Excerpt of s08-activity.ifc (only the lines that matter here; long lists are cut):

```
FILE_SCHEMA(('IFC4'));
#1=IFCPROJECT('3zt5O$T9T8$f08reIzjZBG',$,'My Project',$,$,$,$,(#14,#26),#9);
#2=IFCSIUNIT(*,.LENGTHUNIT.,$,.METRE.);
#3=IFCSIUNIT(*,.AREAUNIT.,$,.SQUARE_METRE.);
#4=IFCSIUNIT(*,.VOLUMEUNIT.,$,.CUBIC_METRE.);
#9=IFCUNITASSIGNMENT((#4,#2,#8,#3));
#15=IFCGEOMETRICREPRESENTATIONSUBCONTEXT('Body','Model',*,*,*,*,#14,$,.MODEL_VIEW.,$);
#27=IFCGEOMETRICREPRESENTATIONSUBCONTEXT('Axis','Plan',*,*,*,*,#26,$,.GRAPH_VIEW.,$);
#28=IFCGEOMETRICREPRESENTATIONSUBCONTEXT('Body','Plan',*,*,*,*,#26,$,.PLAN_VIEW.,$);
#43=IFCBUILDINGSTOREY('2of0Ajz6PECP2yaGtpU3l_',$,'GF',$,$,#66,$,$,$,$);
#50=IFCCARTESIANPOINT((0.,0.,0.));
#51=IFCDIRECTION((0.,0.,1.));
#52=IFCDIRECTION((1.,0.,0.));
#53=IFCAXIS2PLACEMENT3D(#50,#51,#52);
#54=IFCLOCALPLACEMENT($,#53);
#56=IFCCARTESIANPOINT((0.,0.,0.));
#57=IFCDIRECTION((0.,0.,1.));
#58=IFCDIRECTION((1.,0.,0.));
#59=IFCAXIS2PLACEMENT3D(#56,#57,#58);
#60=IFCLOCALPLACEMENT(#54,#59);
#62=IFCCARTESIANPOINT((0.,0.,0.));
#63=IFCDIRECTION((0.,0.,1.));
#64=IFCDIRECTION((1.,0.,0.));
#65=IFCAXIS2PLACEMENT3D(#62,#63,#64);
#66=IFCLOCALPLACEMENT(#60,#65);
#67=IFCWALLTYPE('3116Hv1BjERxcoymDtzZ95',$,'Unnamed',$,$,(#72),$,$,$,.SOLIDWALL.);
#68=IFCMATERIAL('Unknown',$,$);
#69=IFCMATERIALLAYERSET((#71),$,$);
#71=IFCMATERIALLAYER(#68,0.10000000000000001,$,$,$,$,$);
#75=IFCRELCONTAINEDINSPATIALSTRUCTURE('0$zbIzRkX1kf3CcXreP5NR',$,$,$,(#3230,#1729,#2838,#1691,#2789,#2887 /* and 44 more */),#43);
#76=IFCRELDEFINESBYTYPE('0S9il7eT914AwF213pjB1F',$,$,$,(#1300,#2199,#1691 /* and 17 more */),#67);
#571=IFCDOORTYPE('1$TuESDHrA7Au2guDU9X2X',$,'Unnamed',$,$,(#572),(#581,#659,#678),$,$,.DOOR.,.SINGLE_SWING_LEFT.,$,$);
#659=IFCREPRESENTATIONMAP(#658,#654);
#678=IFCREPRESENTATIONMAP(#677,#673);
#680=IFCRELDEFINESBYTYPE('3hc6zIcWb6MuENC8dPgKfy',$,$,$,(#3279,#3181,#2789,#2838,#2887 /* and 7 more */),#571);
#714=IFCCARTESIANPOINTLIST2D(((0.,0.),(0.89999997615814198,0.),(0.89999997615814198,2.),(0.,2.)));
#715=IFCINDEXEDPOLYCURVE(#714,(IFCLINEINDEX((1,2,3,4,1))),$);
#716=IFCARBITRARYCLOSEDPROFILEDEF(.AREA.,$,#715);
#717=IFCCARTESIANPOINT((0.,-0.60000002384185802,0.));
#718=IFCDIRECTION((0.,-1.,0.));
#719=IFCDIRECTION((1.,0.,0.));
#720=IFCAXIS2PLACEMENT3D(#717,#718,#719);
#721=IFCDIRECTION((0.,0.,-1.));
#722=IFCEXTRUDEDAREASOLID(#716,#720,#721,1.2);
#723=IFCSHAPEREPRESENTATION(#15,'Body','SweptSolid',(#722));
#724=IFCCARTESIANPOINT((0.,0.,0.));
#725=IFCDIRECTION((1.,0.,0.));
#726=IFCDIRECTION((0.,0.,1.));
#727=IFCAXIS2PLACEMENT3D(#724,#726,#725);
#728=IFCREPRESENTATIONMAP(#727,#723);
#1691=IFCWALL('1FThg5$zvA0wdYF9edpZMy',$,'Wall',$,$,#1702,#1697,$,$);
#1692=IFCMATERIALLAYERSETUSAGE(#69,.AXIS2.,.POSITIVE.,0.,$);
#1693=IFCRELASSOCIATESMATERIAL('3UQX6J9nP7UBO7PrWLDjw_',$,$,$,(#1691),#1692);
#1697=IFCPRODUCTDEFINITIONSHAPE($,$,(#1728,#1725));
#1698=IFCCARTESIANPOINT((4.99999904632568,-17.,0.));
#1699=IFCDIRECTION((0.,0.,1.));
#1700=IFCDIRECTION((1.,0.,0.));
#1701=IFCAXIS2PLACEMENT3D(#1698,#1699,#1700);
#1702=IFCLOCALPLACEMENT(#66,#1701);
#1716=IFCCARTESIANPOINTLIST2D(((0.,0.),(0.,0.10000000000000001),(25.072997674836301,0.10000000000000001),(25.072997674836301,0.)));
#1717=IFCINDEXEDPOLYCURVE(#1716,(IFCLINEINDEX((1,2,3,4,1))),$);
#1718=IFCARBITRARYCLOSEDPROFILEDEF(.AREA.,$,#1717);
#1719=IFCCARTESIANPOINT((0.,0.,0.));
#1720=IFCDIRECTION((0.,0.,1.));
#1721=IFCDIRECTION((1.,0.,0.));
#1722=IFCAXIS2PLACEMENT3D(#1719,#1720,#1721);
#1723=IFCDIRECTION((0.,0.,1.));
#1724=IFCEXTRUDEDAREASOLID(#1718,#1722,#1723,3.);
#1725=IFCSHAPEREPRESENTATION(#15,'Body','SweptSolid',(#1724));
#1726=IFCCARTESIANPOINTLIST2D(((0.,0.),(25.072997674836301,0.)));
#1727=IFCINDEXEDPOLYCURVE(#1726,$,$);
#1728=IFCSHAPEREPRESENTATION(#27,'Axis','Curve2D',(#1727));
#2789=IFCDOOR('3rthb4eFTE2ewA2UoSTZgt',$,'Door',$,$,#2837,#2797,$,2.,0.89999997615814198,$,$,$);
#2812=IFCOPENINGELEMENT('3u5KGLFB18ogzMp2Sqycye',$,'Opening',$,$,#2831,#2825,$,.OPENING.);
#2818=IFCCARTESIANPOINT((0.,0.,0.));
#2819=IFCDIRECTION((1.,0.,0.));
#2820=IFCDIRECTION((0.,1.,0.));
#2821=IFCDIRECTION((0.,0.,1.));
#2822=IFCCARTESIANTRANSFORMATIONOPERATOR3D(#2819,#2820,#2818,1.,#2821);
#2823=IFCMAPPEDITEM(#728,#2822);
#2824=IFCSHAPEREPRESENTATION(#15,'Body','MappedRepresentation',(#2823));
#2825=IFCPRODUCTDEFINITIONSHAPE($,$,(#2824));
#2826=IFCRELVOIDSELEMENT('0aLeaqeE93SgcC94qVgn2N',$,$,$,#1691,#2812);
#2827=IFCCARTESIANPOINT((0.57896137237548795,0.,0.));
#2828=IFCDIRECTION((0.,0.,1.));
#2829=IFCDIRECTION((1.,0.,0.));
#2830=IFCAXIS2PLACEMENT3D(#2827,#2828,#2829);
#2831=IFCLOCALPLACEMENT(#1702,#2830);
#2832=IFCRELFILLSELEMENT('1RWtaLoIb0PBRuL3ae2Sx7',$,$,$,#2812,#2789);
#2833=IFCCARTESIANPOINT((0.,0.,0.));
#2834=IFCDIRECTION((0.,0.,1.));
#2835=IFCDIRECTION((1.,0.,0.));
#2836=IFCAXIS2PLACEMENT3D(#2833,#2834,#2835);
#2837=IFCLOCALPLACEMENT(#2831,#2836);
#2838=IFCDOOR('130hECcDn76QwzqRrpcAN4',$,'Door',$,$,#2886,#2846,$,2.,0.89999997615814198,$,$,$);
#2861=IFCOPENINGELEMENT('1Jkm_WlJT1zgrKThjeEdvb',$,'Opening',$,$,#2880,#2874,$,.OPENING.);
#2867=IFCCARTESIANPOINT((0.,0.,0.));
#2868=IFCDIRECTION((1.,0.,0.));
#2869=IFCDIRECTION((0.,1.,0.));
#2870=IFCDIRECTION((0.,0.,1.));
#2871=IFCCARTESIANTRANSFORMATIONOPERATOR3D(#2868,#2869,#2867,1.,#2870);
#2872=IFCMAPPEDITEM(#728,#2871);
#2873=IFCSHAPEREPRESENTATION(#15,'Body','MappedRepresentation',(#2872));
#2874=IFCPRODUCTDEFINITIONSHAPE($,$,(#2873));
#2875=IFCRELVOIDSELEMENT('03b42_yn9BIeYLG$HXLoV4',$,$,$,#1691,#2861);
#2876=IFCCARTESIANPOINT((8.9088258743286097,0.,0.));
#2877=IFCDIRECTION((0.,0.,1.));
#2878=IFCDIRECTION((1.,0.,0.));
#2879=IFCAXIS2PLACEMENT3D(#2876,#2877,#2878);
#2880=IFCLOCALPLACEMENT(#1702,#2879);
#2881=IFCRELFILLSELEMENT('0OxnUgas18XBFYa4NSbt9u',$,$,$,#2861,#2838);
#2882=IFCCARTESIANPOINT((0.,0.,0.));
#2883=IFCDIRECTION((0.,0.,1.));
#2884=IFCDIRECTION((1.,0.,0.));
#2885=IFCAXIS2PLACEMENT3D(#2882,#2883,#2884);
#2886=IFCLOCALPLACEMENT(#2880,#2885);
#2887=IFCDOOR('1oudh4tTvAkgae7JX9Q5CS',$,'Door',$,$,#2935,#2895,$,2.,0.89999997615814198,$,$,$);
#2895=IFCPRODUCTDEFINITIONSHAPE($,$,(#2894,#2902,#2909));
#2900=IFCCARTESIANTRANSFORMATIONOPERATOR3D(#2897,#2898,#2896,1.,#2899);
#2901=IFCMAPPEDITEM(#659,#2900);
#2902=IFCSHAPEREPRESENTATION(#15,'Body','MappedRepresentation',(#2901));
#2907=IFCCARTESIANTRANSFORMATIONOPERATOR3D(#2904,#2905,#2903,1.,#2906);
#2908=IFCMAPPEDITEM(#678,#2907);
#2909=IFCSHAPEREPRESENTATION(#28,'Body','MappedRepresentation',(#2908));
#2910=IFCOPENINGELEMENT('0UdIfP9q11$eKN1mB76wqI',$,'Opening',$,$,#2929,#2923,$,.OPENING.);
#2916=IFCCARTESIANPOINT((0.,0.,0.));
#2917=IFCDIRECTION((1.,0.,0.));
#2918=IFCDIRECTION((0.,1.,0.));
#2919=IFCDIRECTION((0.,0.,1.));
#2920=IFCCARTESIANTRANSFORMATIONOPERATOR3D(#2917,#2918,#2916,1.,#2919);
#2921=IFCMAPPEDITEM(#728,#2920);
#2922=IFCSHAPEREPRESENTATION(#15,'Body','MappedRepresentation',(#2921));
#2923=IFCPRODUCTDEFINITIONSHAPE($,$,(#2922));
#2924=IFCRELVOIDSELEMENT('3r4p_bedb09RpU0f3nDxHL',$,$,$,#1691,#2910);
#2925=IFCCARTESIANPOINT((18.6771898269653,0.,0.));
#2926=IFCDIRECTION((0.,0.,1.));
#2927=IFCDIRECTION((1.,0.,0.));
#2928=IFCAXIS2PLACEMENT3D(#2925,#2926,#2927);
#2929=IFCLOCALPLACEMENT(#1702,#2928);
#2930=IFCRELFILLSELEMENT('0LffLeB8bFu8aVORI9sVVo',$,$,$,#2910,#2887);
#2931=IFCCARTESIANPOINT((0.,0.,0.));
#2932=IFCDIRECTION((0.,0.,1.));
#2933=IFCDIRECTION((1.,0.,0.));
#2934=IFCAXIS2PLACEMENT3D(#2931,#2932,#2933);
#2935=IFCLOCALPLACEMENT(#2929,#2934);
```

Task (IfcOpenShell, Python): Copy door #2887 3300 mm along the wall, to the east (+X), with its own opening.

```python
import ifcopenshell
import ifcopenshell.api.feature
import ifcopenshell.api.geometry
import ifcopenshell.api.root
import ifcopenshell.geom
import ifcopenshell.util.element
import ifcopenshell.util.placement
import ifcopenshell.util.shape

model = ifcopenshell.open("s08-activity.ifc")
settings = ifcopenshell.geom.settings()


def volume(element):
    """Net volume in cubic metres, openings subtracted."""
    shape = ifcopenshell.geom.create_shape(settings, element)
    return ifcopenshell.util.shape.get_volume(shape.geometry)


door = model.by_guid("1oudh4tTvAkgae7JX9Q5CS")
opening = door.FillsVoids[0].RelatingOpeningElement
wall = opening.VoidsElements[0].RelatingBuildingElement
before = volume(wall)
shift = ifcopenshell.util.placement.get_local_placement(wall.ObjectPlacement)[:3, 0] * 3.3

# copy_class copies the void relationship, type, container and properties, but no geometry.
new_opening = ifcopenshell.api.root.copy_class(model, product=opening)
new_opening.Representation = ifcopenshell.util.element.copy_deep(
    model, opening.Representation, exclude=["IfcGeometricRepresentationContext", "IfcRepresentationMap"]
)
new_door = ifcopenshell.api.root.copy_class(model, product=door)
new_door.Representation = ifcopenshell.util.element.copy_deep(
    model, door.Representation, exclude=["IfcGeometricRepresentationContext", "IfcRepresentationMap"]
)
ifcopenshell.api.feature.add_filling(model, opening=new_opening, element=new_door)

for old, new in ((opening, new_opening), (door, new_door)):
    matrix = ifcopenshell.util.placement.get_local_placement(old.ObjectPlacement)
    matrix[:3, 3] += shift
    ifcopenshell.api.geometry.edit_object_placement(model, product=new, matrix=matrix, is_si=False)

after = volume(wall)

print(f"wall volume {before:.3f} -> {after:.3f} m3")

model.write("s08-activity_updated.ifc")
```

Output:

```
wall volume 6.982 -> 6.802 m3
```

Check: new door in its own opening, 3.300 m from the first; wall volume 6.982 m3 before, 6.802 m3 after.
